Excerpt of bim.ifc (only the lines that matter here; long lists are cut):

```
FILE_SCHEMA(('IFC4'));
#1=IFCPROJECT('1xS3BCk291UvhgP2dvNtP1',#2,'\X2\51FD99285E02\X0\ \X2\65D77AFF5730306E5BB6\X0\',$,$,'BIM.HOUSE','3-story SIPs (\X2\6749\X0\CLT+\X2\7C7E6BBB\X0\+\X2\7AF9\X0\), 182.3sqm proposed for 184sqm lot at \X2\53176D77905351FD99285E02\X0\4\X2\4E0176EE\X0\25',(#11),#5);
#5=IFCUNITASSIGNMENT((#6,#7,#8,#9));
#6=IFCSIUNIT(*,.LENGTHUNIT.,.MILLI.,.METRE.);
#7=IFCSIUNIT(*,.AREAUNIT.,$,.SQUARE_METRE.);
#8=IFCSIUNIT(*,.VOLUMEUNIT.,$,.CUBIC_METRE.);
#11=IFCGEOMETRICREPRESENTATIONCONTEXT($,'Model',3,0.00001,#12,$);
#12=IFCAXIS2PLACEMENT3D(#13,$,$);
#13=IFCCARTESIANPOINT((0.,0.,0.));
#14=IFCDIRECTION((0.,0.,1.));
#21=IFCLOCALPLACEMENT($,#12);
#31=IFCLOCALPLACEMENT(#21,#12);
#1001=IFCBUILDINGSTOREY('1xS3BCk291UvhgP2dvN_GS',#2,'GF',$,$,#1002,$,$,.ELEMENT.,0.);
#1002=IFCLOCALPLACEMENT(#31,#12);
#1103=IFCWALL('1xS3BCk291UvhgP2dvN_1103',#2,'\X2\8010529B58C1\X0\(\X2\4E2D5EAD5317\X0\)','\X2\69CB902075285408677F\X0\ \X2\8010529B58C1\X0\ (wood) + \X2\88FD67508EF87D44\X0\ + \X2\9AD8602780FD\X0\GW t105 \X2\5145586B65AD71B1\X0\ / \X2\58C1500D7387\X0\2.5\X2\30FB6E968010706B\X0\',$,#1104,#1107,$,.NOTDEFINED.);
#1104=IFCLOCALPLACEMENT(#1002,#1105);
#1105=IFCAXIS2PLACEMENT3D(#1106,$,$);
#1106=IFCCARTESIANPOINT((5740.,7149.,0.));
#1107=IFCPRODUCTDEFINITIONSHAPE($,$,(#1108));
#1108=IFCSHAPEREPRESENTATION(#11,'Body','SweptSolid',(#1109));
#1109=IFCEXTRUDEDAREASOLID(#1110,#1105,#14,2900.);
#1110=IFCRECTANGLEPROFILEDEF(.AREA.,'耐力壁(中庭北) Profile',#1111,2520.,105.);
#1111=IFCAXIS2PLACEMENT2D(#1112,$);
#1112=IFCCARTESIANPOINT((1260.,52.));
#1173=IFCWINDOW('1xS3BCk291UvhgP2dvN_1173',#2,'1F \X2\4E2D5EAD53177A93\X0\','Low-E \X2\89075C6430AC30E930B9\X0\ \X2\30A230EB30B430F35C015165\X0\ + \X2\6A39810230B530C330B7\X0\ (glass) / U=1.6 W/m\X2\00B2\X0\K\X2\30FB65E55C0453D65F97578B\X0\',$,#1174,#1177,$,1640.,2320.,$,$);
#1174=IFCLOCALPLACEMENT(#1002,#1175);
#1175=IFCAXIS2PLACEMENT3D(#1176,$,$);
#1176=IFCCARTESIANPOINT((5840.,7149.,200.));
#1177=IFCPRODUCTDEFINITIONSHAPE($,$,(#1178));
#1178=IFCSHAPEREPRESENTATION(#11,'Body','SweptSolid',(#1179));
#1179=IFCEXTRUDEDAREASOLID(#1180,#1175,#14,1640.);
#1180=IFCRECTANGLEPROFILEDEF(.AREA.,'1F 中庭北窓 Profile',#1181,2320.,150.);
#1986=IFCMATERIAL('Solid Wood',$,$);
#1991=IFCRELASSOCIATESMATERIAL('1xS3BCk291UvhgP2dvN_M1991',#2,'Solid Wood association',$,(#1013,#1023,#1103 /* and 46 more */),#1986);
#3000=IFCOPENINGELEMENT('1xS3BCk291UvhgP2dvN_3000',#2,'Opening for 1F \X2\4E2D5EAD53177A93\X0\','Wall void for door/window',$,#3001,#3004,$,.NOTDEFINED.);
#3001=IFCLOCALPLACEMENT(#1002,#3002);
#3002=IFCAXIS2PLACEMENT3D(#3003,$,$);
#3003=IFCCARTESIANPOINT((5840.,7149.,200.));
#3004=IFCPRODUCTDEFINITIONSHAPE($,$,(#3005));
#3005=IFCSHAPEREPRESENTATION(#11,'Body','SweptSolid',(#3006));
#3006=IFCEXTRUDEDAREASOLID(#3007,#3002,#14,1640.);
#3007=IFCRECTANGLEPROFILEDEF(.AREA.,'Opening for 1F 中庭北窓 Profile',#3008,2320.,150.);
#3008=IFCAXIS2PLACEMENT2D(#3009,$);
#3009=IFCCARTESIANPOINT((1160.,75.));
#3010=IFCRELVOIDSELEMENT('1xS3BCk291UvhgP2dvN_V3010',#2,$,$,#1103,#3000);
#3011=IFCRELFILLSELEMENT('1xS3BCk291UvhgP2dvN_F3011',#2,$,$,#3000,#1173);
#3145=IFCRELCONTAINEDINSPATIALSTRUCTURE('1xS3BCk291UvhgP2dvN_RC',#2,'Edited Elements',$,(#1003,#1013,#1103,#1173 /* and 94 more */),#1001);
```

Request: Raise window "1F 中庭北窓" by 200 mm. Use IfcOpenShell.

```python
import numpy as np
import ifcopenshell
import ifcopenshell.api.geometry
import ifcopenshell.util.placement
import ifcopenshell.util.unit

model = ifcopenshell.open("bim.ifc")
unit_scale = ifcopenshell.util.unit.calculate_unit_scale(model)

window = model.by_guid("1xS3BCk291UvhgP2dvN_1173")
opening = window.FillsVoids[0].RelatingOpeningElement
dz = 200.0

shift = np.array([0.0, 0.0, dz])
# The window is not placed relative to its opening, so move both.
for product in (opening, window):
    matrix = ifcopenshell.util.placement.get_local_placement(product.ObjectPlacement)
    matrix[:3, 3] += shift
    ifcopenshell.api.geometry.edit_object_placement(model, product=product, matrix=matrix, is_si=False)

print(f"moved by {dz * unit_scale:+.3f} m")

model.write("bim_edited.ifc")
```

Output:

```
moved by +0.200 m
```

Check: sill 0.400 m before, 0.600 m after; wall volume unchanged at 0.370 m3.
